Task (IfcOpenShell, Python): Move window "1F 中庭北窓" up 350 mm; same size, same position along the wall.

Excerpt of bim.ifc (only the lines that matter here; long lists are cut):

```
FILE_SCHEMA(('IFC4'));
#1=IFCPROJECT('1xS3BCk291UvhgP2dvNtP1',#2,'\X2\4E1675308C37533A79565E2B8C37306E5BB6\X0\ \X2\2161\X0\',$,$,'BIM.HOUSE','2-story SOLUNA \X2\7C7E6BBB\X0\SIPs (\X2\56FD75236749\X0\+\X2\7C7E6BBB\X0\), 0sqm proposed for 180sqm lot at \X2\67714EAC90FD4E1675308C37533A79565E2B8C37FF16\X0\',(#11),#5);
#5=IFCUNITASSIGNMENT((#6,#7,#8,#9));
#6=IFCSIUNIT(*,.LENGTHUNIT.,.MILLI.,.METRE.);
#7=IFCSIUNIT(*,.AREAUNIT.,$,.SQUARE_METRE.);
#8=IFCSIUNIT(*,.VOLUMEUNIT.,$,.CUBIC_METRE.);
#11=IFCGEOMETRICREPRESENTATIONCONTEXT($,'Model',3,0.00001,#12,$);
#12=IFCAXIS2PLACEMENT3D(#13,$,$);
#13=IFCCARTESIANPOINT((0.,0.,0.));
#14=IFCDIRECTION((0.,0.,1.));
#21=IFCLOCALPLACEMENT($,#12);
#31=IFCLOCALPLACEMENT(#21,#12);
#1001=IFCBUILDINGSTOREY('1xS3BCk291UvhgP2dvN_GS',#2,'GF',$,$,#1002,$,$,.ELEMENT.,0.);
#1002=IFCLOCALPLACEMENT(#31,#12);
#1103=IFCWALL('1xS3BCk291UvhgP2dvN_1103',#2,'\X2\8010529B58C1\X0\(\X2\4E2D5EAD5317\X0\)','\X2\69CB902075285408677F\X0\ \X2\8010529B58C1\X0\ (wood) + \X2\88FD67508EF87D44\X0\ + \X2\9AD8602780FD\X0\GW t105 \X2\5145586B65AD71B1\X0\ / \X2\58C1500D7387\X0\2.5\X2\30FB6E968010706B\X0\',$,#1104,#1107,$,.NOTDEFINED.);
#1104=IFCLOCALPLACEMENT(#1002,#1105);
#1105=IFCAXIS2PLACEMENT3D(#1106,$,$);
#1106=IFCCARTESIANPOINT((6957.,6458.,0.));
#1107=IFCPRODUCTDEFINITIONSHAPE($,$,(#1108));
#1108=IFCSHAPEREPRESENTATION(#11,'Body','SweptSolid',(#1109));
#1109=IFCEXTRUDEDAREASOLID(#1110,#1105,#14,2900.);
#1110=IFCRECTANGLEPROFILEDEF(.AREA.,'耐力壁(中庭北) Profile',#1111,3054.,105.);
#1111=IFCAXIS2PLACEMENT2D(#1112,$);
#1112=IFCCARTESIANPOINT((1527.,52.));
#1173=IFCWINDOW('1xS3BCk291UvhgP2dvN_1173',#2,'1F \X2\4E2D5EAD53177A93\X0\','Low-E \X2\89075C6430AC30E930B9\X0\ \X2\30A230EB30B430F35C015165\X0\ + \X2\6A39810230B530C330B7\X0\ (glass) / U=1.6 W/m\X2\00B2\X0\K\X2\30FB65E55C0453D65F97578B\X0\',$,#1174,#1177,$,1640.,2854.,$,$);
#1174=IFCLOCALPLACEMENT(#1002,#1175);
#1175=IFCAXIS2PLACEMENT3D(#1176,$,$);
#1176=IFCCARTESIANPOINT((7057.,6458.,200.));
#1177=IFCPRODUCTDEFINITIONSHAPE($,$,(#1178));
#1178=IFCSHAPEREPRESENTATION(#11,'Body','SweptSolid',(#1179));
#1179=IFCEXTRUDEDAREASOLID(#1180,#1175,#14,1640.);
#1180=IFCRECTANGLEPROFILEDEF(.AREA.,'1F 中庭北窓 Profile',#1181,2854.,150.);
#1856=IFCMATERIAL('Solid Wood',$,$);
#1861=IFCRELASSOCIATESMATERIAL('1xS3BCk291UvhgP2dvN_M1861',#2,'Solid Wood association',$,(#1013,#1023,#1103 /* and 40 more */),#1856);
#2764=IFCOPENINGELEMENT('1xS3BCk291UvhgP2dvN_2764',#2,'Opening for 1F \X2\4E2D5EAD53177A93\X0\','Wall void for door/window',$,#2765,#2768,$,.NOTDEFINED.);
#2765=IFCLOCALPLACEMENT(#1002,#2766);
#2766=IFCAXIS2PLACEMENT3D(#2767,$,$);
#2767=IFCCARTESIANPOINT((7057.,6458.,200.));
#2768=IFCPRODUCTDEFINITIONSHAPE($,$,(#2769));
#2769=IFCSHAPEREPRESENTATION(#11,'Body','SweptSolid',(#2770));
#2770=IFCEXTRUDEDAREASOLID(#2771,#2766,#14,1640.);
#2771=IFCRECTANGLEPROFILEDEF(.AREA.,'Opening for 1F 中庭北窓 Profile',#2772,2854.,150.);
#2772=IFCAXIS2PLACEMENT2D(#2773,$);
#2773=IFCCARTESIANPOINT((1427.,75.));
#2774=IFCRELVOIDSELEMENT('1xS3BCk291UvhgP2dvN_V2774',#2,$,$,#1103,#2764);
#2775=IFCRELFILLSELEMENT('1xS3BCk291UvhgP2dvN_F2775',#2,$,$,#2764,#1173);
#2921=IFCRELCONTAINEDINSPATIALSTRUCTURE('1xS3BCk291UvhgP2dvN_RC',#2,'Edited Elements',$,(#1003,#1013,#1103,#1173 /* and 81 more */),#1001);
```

```python
import numpy as np
import ifcopenshell
import ifcopenshell.api.geometry
import ifcopenshell.util.placement
import ifcopenshell.util.unit

model = ifcopenshell.open("bim.ifc")
unit_scale = ifcopenshell.util.unit.calculate_unit_scale(model)

window = model.by_guid("1xS3BCk291UvhgP2dvN_1173")
opening = window.FillsVoids[0].RelatingOpeningElement
dz = 350.0

shift = np.array([0.0, 0.0, dz])
# The window is not placed relative to its opening, so move both.
for product in (opening, window):
    matrix = ifcopenshell.util.placement.get_local_placement(product.ObjectPlacement)
    matrix[:3, 3] += shift
    ifcopenshell.api.geometry.edit_object_placement(model, product=product, matrix=matrix, is_si=False)

print(f"moved by {dz * unit_scale:+.3f} m")

model.write("bim_rev.ifc")
```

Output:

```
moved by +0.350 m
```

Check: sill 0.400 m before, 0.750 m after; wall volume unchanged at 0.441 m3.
